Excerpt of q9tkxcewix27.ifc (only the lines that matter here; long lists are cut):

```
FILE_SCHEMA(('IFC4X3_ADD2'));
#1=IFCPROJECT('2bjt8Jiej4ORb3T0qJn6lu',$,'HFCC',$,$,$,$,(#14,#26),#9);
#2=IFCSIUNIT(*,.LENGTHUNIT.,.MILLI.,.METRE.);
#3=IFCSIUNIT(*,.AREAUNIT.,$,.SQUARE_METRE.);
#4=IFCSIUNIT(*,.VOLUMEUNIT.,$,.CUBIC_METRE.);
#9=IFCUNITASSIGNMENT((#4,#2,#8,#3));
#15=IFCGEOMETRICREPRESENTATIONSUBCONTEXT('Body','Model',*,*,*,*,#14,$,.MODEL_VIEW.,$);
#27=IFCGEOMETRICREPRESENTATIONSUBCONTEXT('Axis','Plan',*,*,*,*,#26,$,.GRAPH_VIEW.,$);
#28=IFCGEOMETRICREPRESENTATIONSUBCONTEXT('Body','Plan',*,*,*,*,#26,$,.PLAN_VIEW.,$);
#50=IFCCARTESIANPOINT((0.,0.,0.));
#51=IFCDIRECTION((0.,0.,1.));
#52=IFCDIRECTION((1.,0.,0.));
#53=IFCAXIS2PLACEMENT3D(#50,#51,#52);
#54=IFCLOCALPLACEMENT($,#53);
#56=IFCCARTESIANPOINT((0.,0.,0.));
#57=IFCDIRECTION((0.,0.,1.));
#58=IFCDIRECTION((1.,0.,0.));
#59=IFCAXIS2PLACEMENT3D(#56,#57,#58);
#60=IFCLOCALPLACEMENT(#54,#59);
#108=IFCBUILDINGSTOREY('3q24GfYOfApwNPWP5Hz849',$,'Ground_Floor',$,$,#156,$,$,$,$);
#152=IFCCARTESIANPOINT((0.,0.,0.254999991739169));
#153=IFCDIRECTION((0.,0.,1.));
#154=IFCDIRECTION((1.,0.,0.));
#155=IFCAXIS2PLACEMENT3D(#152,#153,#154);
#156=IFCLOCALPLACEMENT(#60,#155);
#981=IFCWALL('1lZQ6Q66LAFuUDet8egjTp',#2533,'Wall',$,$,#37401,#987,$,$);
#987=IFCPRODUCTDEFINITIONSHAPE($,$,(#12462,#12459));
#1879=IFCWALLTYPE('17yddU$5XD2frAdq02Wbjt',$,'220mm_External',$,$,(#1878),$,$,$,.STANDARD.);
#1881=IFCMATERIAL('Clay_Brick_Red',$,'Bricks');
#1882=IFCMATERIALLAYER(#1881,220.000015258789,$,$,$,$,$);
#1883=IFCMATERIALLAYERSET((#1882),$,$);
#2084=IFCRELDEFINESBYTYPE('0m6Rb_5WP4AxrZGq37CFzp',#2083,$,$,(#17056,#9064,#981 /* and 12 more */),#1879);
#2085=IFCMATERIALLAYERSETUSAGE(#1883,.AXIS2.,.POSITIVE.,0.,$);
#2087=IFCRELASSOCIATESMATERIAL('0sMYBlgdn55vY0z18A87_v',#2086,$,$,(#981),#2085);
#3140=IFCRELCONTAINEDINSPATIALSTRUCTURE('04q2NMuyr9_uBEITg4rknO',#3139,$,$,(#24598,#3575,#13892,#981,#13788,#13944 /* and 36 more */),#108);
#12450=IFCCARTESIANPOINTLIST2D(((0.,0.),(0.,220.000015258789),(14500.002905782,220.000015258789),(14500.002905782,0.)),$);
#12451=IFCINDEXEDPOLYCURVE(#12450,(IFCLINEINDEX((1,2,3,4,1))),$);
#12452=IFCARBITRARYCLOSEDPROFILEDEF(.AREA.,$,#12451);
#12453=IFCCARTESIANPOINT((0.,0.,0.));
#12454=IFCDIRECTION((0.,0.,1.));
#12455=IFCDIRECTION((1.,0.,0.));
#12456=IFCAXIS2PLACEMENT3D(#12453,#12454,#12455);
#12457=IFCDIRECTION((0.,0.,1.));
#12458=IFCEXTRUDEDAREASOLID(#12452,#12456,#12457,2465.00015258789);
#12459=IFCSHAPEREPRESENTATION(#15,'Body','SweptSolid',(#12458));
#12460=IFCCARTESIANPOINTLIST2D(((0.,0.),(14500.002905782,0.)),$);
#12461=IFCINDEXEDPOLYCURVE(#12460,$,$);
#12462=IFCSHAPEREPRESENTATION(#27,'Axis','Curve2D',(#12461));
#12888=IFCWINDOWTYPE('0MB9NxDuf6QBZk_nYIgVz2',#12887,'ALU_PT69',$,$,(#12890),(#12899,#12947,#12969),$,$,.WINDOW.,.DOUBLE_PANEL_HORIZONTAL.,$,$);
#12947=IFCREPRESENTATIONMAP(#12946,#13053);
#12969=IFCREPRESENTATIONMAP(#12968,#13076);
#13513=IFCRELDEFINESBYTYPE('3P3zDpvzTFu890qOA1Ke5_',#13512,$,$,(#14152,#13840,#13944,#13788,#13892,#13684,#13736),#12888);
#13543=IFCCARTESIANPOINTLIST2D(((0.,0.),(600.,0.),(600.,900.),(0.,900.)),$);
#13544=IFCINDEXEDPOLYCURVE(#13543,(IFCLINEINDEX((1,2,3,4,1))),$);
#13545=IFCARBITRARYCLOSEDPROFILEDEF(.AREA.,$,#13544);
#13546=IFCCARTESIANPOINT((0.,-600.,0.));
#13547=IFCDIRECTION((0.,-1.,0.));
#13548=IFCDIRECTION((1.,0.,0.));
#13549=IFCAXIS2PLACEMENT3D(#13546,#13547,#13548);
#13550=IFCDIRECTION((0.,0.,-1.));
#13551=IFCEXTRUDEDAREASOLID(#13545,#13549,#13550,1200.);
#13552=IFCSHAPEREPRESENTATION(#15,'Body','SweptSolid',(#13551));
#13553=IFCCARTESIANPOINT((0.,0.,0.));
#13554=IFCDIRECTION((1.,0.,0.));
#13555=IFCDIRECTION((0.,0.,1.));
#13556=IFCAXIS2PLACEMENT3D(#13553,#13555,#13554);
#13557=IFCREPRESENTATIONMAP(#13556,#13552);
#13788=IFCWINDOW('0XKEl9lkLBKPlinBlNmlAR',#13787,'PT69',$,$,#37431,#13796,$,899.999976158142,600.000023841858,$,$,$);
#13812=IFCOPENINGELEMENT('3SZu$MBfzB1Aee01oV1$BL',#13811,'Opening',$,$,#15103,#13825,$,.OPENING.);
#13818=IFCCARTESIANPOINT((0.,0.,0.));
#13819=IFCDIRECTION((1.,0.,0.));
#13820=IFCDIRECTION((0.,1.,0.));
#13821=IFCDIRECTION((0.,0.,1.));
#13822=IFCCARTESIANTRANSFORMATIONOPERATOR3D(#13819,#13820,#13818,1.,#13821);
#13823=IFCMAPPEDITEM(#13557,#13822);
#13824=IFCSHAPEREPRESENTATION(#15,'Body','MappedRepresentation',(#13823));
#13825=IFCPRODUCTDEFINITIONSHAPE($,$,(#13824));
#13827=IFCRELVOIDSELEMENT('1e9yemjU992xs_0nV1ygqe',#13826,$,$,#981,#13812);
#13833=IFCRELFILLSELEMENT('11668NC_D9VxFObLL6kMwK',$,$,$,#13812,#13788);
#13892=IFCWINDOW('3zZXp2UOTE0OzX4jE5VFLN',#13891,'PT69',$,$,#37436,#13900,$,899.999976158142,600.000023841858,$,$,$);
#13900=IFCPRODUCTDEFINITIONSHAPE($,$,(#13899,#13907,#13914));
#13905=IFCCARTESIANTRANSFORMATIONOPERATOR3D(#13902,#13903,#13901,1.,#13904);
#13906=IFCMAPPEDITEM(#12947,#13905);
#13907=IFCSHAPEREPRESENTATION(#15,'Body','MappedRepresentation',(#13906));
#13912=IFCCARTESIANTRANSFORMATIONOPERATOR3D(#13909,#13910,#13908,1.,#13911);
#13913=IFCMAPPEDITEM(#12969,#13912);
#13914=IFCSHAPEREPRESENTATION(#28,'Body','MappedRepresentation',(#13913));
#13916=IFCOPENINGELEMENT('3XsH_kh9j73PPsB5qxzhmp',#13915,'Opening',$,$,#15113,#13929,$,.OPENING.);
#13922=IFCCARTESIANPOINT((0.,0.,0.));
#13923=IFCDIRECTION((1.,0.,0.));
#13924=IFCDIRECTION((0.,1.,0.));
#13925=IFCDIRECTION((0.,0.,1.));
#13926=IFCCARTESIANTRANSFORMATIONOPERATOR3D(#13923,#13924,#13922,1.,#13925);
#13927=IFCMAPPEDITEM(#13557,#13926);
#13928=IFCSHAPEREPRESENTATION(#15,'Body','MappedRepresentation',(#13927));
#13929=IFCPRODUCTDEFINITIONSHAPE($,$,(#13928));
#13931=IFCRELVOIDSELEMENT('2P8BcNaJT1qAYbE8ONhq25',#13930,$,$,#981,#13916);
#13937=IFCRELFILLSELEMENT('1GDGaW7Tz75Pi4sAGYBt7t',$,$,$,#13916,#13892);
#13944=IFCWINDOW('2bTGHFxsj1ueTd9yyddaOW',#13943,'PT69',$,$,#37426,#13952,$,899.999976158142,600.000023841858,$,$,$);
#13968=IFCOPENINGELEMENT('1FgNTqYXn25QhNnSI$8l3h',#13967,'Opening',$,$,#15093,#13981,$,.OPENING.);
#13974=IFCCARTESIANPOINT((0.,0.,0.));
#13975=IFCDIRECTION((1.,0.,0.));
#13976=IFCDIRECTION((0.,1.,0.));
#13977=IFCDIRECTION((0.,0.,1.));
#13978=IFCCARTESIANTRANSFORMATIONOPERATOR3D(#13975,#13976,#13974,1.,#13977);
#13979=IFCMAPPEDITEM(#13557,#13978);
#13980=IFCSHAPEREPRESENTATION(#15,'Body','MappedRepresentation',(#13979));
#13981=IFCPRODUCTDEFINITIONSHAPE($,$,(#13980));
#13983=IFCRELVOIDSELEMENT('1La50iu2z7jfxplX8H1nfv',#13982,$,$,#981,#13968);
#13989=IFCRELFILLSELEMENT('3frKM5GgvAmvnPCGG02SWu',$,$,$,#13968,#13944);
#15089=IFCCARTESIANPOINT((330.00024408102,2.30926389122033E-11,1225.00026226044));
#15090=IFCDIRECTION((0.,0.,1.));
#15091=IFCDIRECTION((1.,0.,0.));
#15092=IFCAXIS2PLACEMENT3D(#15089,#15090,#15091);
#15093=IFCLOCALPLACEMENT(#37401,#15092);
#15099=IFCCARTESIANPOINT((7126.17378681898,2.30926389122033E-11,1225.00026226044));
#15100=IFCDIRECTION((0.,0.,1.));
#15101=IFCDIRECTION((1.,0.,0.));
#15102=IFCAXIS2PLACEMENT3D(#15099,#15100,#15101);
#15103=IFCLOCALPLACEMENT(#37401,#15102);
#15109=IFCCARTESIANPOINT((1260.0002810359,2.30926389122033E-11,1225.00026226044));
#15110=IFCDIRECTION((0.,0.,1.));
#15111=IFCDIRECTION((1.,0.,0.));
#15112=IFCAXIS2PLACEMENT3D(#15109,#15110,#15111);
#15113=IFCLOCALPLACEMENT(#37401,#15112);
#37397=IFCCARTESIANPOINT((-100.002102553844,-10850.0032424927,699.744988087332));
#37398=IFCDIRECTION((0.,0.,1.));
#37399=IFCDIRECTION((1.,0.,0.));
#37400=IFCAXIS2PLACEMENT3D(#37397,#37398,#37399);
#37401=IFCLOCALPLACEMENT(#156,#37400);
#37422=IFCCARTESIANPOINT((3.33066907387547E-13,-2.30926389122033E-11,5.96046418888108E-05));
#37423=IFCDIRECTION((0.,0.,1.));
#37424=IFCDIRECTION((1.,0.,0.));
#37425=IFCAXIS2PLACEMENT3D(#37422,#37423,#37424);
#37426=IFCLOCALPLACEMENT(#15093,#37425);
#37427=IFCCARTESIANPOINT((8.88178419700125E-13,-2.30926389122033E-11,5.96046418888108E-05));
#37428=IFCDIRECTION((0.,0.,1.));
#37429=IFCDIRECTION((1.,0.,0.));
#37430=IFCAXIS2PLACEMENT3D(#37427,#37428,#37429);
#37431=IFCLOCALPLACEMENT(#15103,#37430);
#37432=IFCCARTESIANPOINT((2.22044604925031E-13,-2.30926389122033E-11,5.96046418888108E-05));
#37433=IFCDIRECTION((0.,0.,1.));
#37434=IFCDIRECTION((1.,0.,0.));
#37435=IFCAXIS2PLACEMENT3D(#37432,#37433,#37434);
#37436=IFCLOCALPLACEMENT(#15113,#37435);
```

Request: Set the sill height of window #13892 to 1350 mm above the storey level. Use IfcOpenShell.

```python
import numpy as np
import ifcopenshell
import ifcopenshell.api.geometry
import ifcopenshell.geom
import ifcopenshell.util.element
import ifcopenshell.util.placement
import ifcopenshell.util.shape
import ifcopenshell.util.unit

model = ifcopenshell.open("q9tkxcewix27.ifc")
unit_scale = ifcopenshell.util.unit.calculate_unit_scale(model)

window = model.by_guid("3zZXp2UOTE0OzX4jE5VFLN")
opening = window.FillsVoids[0].RelatingOpeningElement
storey = ifcopenshell.util.element.get_container(window, ifc_class="IfcBuildingStorey")
level = ifcopenshell.util.placement.get_local_placement(storey.ObjectPlacement)[2, 3]

# The opening's origin need not be at the sill, so measure its lowest point.
shape = ifcopenshell.geom.create_shape(ifcopenshell.geom.settings(), opening)
bottom = ifcopenshell.util.shape.get_shape_bottom_elevation(shape, shape.geometry) / unit_scale
dz = level + 1.35 / unit_scale - bottom

shift = np.array([0.0, 0.0, dz])
# The window is placed relative to its opening, so it follows when the opening moves.
matrix = ifcopenshell.util.placement.get_local_placement(opening.ObjectPlacement)
matrix[:3, 3] += shift
ifcopenshell.api.geometry.edit_object_placement(
    model, product=opening, matrix=matrix, is_si=False, should_transform_children=True
)

print(f"moved by {dz * unit_scale:+.3f} m")

model.write("q9tkxcewix27_updated.ifc")
```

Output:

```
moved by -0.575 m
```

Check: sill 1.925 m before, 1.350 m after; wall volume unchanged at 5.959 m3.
